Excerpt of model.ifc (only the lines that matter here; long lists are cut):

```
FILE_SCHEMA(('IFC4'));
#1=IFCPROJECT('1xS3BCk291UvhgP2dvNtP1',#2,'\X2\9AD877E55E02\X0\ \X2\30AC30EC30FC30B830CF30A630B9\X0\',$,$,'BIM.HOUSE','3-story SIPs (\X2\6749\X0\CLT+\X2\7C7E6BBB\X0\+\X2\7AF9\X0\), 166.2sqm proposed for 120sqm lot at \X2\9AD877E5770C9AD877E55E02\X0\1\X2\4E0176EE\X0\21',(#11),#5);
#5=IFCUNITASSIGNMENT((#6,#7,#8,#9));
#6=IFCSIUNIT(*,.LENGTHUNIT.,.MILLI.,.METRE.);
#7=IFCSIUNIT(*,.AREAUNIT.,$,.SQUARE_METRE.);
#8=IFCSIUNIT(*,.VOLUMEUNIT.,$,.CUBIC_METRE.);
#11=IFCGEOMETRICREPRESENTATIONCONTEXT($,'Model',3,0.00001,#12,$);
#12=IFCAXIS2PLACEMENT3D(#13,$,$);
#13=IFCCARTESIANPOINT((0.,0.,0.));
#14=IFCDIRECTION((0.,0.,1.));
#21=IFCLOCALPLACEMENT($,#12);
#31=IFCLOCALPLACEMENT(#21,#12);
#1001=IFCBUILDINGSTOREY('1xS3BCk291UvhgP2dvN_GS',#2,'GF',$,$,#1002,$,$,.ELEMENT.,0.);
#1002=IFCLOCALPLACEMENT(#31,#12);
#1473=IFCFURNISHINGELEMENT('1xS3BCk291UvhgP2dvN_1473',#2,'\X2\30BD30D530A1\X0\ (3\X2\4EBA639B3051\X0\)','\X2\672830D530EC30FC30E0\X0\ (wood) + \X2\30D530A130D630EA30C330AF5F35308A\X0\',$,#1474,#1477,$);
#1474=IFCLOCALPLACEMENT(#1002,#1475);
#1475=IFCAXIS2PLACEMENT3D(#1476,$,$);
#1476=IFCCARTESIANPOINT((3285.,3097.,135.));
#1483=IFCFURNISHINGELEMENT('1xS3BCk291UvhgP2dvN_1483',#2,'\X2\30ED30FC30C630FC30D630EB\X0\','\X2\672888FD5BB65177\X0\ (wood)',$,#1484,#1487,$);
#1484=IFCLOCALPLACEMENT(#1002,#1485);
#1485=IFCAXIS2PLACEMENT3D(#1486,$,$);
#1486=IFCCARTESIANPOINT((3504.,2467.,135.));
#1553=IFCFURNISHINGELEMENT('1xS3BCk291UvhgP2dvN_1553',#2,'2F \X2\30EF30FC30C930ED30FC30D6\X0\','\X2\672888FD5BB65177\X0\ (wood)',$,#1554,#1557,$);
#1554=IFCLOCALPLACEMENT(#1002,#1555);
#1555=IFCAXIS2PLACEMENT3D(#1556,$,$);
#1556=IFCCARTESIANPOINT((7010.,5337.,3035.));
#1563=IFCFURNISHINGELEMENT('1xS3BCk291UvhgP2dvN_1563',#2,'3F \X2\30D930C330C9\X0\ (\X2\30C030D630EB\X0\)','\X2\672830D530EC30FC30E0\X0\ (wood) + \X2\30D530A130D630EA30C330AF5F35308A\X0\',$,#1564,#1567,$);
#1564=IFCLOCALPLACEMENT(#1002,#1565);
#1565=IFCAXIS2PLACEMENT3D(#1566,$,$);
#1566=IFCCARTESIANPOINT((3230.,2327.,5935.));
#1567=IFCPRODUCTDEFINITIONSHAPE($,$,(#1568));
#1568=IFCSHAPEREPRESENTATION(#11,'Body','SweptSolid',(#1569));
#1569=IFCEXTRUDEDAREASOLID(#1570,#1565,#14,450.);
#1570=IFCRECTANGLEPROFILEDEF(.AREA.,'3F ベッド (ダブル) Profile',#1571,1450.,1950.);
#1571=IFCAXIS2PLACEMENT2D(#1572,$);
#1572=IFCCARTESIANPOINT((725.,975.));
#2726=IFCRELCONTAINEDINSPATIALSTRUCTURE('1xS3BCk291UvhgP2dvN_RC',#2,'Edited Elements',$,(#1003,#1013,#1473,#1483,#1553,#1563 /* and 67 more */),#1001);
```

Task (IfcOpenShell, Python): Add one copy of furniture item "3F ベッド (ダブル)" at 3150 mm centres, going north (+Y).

```python
import numpy as np
import ifcopenshell
import ifcopenshell.api.geometry
import ifcopenshell.api.root
import ifcopenshell.util.element
import ifcopenshell.util.placement
import ifcopenshell.util.unit

model = ifcopenshell.open("model.ifc")
unit_scale = ifcopenshell.util.unit.calculate_unit_scale(model)


def reuse_history(source, copy):
    """copy_class also copies each property set's owner history, people and application; keep the originals."""
    for rel in copy.IsDefinedBy:
        if rel.is_a("IfcRelDefinesByProperties") and (history := rel.RelatingPropertyDefinition.OwnerHistory):
            rel.RelatingPropertyDefinition.OwnerHistory = source.OwnerHistory
            ifcopenshell.util.element.remove_deep2(model, history)


source = model.by_id(1563)
base = ifcopenshell.util.placement.get_local_placement(source.ObjectPlacement)
step = np.array([0.0, 1.0, 0.0]) * 3.15 / unit_scale

for i in range(1, 2):
    copy = ifcopenshell.api.root.copy_class(model, product=source)
    copy.Representation = ifcopenshell.util.element.copy_deep(
        model, source.Representation, exclude=["IfcGeometricRepresentationContext", "IfcRepresentationMap"]
    )
    reuse_history(source, copy)
    matrix = base.copy()
    matrix[:3, 3] += i * step
    print("added at", matrix[:3, 3].round(3) + 0.0)
    ifcopenshell.api.geometry.edit_object_placement(model, product=copy, matrix=matrix, is_si=False)

model.write("model_edited.ifc")
```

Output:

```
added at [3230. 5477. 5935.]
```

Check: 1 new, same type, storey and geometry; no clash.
